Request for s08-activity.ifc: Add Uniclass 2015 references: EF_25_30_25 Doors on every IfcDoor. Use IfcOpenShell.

First a look at what the model holds.

```python
import ifcopenshell

model = ifcopenshell.open("s08-activity.ifc")
print(model.schema)
print("classifications:", [c.Name for c in model.by_type("IfcClassification")])
for ifc_class in ("IfcDoor", "IfcRoof", "IfcStair", "IfcWall", "IfcWindow"):
    print(ifc_class, len(model.by_type(ifc_class)))
```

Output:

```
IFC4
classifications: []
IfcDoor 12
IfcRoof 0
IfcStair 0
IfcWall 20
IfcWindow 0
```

```python
import ifcopenshell
import ifcopenshell.api.classification

model = ifcopenshell.open("s08-activity.ifc")

system = ifcopenshell.api.classification.add_classification(model, classification="Uniclass 2015")

codes = {
    "IfcDoor": ("EF_25_30_25", "Doors"),
}
for ifc_class, (code, name) in codes.items():
    products = model.by_type(ifc_class)
    ifcopenshell.api.classification.add_reference(
        model, products=products, classification=system, identification=code, name=name
    )
    print(code, len(products))

model.write("s08-activity_updated.ifc")
```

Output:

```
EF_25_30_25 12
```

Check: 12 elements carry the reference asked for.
